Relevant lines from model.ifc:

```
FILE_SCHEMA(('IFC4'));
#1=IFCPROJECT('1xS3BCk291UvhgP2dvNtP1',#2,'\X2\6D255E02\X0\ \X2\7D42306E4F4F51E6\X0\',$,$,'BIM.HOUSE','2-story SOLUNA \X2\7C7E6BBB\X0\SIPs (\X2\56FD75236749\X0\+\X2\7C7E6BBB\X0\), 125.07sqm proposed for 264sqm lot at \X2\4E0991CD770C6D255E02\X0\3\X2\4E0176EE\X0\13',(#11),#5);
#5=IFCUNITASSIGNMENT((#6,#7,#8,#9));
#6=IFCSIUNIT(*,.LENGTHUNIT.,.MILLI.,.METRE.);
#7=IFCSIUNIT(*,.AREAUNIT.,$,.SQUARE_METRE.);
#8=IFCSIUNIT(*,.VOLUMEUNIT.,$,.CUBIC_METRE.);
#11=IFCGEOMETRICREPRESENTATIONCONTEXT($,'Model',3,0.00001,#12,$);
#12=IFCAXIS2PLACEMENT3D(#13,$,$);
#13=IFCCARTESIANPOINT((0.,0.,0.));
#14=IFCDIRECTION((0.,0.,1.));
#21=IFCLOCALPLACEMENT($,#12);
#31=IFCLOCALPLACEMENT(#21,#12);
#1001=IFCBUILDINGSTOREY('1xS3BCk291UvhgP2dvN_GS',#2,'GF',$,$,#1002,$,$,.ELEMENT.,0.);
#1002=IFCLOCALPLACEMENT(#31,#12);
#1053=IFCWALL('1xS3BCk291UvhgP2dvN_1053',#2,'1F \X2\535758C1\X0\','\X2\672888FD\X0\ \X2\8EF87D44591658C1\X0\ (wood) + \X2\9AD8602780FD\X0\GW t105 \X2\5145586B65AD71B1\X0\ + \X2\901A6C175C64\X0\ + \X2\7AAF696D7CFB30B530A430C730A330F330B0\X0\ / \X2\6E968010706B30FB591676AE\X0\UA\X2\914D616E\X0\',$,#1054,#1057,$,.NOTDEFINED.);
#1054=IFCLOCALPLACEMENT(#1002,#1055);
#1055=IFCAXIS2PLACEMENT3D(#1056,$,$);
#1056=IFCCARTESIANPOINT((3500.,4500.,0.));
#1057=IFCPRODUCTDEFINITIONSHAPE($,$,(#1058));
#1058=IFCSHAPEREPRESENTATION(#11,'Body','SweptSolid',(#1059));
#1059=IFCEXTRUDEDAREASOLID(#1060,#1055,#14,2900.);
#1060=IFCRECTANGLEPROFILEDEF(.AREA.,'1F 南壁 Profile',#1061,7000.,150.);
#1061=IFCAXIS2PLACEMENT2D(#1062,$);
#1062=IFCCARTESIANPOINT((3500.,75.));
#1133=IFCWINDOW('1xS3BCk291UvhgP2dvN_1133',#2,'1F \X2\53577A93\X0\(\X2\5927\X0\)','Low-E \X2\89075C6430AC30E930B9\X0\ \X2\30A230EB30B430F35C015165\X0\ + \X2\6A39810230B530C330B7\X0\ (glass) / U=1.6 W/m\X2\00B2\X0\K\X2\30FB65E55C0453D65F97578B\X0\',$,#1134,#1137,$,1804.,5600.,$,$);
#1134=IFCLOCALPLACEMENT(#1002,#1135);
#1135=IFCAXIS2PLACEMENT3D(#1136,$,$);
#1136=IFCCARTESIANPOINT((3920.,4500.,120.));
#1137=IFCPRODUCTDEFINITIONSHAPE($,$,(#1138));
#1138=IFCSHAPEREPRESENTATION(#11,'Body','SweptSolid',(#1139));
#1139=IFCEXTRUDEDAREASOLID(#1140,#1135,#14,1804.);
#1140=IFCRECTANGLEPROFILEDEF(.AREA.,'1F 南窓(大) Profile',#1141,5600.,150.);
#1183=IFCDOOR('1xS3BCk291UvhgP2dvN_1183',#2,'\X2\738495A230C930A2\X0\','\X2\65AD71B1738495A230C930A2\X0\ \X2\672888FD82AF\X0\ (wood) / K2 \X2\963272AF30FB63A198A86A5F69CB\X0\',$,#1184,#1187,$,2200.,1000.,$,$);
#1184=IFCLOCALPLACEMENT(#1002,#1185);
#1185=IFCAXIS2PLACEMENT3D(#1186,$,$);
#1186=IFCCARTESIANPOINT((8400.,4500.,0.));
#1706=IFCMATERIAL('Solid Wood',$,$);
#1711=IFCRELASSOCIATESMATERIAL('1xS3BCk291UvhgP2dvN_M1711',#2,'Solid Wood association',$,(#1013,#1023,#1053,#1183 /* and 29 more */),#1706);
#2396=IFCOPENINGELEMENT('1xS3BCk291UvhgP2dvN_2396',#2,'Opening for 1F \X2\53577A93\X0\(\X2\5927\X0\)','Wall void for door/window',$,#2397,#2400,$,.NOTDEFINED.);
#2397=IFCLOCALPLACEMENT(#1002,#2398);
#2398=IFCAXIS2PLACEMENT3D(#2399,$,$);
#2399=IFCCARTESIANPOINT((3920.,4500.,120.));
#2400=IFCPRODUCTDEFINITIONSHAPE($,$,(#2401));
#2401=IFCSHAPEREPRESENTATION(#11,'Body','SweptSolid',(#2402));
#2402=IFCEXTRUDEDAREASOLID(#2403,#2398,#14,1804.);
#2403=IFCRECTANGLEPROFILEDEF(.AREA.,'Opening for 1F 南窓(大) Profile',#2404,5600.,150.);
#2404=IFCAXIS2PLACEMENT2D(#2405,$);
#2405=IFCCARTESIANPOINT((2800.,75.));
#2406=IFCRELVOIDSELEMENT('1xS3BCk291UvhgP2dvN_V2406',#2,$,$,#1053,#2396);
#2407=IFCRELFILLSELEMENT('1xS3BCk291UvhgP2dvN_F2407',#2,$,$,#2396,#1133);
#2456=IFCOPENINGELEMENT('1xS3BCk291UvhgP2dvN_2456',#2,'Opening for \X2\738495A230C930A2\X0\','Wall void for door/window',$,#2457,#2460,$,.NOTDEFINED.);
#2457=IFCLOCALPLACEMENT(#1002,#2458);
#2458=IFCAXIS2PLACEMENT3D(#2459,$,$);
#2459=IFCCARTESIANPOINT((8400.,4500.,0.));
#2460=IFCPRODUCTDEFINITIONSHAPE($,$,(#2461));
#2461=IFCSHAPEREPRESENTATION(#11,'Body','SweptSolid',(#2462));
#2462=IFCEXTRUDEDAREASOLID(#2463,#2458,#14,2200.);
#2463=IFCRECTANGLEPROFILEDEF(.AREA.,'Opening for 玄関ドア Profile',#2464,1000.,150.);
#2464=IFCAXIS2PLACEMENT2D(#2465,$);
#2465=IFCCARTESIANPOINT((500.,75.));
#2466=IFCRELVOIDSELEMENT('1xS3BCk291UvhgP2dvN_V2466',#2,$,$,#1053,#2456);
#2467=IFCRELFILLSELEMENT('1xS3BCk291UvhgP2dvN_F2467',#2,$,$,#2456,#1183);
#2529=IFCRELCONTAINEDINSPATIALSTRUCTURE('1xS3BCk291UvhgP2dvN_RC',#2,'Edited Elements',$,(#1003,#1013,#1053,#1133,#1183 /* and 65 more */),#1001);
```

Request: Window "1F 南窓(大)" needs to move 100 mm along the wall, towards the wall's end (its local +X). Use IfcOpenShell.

```python
import ifcopenshell
import ifcopenshell.api.geometry
import ifcopenshell.util.placement

model = ifcopenshell.open("model.ifc")

window = model.by_guid("1xS3BCk291UvhgP2dvN_1133")
opening = window.FillsVoids[0].RelatingOpeningElement
wall = opening.VoidsElements[0].RelatingBuildingElement

wall_matrix = ifcopenshell.util.placement.get_local_placement(wall.ObjectPlacement)
shift = wall_matrix[:3, 0] * 100.0
before = ifcopenshell.util.placement.get_local_placement(window.ObjectPlacement)[:3, 3].copy()

# The window is not placed relative to its opening, so move both.
for product in (opening, window):
    matrix = ifcopenshell.util.placement.get_local_placement(product.ObjectPlacement)
    matrix[:3, 3] += shift
    ifcopenshell.api.geometry.edit_object_placement(model, product=product, matrix=matrix, is_si=False)

after = ifcopenshell.util.placement.get_local_placement(window.ObjectPlacement)[:3, 3]
print("window moved by", (after - before).round(3) + 0.0)

model.write("model_updated.ifc")
```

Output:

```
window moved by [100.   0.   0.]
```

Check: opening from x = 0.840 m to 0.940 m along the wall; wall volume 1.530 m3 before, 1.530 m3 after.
